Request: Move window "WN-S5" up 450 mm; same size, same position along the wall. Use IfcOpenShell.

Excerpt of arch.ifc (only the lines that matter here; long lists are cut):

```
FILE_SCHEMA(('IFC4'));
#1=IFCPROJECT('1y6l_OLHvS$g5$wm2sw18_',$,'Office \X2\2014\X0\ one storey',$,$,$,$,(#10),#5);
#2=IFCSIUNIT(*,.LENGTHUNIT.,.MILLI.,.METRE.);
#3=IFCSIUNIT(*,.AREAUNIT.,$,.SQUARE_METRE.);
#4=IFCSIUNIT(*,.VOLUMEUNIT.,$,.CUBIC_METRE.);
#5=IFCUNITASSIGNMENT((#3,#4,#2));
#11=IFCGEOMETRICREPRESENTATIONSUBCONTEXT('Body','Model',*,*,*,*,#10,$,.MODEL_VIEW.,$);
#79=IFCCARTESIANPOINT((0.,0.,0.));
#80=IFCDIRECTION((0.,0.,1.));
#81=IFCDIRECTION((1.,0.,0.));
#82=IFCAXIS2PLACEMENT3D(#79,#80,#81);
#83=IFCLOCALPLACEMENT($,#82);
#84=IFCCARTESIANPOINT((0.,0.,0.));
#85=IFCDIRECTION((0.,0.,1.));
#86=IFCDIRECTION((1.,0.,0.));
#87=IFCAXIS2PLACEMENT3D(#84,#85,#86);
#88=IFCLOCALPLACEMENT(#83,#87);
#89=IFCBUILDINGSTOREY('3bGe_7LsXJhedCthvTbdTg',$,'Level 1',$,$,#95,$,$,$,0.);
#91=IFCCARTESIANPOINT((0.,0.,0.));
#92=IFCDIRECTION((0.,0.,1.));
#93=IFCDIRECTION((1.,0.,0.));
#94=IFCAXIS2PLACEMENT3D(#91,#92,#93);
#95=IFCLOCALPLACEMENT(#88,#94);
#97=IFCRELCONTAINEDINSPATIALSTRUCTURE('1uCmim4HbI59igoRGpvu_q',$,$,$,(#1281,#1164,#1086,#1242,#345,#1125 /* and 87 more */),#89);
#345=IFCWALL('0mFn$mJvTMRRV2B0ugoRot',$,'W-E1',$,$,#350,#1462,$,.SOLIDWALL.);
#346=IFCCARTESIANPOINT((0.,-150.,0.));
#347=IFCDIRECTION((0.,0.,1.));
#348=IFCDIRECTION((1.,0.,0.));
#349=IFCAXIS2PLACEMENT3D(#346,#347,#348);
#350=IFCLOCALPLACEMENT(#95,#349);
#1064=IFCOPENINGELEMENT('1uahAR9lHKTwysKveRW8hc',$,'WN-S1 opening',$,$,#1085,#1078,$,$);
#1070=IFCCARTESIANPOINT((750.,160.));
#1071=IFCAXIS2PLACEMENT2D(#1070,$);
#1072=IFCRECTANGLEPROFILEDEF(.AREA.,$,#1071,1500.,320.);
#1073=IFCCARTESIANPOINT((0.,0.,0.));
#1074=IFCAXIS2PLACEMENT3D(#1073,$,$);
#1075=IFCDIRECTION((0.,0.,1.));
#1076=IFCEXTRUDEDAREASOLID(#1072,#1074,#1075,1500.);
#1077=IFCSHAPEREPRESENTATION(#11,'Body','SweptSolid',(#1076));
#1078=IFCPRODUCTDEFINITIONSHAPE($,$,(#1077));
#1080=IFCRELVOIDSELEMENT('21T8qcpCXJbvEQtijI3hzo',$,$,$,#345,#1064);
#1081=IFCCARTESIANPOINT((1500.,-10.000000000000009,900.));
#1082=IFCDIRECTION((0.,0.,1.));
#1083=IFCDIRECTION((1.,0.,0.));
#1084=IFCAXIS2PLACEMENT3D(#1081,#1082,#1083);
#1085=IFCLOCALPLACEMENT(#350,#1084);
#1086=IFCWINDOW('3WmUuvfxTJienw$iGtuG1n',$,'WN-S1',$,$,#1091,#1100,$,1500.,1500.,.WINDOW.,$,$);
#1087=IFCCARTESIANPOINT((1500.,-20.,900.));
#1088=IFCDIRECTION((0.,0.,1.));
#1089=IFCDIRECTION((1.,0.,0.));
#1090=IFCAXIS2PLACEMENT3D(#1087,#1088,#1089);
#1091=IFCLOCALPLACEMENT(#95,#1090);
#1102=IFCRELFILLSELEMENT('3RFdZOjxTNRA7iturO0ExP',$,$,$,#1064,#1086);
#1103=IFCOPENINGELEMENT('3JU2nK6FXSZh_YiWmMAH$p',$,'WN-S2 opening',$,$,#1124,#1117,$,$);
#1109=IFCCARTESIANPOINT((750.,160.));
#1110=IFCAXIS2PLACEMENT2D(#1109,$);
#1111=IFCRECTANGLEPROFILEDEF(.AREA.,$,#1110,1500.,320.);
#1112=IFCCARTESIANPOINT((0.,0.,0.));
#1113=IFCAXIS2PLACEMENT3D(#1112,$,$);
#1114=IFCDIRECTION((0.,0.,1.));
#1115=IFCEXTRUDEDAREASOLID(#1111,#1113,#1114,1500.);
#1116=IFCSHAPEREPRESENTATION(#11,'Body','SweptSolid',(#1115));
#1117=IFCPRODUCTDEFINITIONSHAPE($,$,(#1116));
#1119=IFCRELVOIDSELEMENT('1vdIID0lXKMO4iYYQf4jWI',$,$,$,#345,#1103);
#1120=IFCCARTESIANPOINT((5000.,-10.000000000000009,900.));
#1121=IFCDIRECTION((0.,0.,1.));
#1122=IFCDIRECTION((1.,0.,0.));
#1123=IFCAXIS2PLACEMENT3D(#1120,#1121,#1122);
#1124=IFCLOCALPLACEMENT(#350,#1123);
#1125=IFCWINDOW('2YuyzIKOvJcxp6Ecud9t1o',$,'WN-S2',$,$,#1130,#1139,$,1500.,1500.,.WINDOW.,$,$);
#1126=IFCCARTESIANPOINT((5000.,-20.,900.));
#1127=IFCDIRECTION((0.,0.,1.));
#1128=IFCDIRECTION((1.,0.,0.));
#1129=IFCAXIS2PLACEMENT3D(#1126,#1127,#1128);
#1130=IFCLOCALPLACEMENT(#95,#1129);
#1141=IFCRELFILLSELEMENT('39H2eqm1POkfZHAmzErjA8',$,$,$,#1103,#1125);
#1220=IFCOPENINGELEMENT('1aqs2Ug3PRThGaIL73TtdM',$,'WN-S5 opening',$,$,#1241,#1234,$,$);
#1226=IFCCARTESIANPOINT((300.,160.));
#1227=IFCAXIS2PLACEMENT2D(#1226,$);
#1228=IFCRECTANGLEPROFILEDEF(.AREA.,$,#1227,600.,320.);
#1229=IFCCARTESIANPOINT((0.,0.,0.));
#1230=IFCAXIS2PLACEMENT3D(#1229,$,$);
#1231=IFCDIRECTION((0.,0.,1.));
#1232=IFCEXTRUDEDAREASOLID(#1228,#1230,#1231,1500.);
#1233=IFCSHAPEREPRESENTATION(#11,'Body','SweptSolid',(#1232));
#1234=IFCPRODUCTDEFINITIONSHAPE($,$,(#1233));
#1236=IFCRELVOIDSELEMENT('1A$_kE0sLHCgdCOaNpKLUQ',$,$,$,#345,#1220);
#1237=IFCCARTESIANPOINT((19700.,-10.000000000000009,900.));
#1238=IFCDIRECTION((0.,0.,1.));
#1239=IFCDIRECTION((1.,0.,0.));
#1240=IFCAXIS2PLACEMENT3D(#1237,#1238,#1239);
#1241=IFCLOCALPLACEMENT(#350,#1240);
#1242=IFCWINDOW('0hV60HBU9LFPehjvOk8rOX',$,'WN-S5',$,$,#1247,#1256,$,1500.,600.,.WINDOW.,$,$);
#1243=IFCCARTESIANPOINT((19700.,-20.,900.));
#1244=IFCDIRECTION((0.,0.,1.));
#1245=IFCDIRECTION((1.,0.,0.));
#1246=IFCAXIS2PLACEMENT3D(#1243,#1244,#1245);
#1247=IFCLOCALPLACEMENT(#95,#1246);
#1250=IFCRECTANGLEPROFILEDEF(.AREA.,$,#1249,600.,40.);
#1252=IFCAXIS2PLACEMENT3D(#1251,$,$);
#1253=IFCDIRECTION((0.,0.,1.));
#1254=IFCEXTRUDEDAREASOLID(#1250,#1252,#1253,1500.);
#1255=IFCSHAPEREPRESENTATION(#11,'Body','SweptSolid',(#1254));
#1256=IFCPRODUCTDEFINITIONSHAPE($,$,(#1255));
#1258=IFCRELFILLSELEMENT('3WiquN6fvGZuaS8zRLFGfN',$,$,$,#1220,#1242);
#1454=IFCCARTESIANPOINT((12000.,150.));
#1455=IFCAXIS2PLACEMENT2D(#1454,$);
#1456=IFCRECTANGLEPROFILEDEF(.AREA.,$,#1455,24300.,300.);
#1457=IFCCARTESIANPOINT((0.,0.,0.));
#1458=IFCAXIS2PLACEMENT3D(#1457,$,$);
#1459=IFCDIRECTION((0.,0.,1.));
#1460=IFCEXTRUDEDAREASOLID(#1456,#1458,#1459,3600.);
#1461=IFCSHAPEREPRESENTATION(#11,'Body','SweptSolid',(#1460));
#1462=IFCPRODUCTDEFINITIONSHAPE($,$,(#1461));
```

```python
import numpy as np
import ifcopenshell
import ifcopenshell.api.geometry
import ifcopenshell.util.placement
import ifcopenshell.util.unit

model = ifcopenshell.open("arch.ifc")
unit_scale = ifcopenshell.util.unit.calculate_unit_scale(model)

window = model.by_guid("0hV60HBU9LFPehjvOk8rOX")
opening = window.FillsVoids[0].RelatingOpeningElement
dz = 0.45 / unit_scale

shift = np.array([0.0, 0.0, dz])
# The window is not placed relative to its opening, so move both.
for product in (opening, window):
    matrix = ifcopenshell.util.placement.get_local_placement(product.ObjectPlacement)
    matrix[:3, 3] += shift
    ifcopenshell.api.geometry.edit_object_placement(model, product=product, matrix=matrix, is_si=False)

print(f"moved by {dz * unit_scale:+.3f} m")

model.write("arch_updated.ifc")
```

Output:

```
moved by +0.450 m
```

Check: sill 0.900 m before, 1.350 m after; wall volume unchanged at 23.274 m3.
